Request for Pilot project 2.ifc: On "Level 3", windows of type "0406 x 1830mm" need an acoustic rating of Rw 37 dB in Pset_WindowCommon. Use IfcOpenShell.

First a look at what the model holds.

```python
import ifcopenshell
import ifcopenshell.util.element

model = ifcopenshell.open("Pilot project 2.ifc")
print(model.schema)
storey = next(s for s in model.by_type("IfcBuildingStorey") if s.Name == "Level 3")
windows = [e for e in ifcopenshell.util.element.get_decomposition(storey) if e.is_a("IfcWindow")]
seen = {}
for e in windows:
    element_type = ifcopenshell.util.element.get_type(e)
    key = (element_type.Name if element_type != e and element_type else None, ifcopenshell.util.element.get_pset(e, "Pset_WindowCommon", "AcousticRating"))
    seen[key] = seen.get(key, 0) + 1
for (name, value), count in sorted(seen.items(), key=str):
    print(count, "x", name, "|", value)
```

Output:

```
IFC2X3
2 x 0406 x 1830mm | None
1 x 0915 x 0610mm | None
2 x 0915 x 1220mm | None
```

```python
import ifcopenshell
import ifcopenshell.api.pset
import ifcopenshell.util.element

model = ifcopenshell.open("Pilot project 2.ifc")

storey = next(s for s in model.by_type("IfcBuildingStorey") if s.Name == "Level 3")
windows = [e for e in ifcopenshell.util.element.get_decomposition(storey) if e.is_a("IfcWindow")]

count = 0
for e in windows:
    element_type = ifcopenshell.util.element.get_type(e)
    if element_type in (None, e) or element_type.Name != "0406 x 1830mm":
        continue
    # add_pset returns the element's existing set when there is one.
    pset = ifcopenshell.api.pset.add_pset(model, product=e, name="Pset_WindowCommon")
    ifcopenshell.api.pset.edit_pset(model, pset=pset, properties={"AcousticRating": "Rw 37 dB"})
    count += 1

print(count, "windows updated")

model.write("Pilot project 2_v2.ifc")
```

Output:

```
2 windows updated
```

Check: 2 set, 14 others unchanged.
